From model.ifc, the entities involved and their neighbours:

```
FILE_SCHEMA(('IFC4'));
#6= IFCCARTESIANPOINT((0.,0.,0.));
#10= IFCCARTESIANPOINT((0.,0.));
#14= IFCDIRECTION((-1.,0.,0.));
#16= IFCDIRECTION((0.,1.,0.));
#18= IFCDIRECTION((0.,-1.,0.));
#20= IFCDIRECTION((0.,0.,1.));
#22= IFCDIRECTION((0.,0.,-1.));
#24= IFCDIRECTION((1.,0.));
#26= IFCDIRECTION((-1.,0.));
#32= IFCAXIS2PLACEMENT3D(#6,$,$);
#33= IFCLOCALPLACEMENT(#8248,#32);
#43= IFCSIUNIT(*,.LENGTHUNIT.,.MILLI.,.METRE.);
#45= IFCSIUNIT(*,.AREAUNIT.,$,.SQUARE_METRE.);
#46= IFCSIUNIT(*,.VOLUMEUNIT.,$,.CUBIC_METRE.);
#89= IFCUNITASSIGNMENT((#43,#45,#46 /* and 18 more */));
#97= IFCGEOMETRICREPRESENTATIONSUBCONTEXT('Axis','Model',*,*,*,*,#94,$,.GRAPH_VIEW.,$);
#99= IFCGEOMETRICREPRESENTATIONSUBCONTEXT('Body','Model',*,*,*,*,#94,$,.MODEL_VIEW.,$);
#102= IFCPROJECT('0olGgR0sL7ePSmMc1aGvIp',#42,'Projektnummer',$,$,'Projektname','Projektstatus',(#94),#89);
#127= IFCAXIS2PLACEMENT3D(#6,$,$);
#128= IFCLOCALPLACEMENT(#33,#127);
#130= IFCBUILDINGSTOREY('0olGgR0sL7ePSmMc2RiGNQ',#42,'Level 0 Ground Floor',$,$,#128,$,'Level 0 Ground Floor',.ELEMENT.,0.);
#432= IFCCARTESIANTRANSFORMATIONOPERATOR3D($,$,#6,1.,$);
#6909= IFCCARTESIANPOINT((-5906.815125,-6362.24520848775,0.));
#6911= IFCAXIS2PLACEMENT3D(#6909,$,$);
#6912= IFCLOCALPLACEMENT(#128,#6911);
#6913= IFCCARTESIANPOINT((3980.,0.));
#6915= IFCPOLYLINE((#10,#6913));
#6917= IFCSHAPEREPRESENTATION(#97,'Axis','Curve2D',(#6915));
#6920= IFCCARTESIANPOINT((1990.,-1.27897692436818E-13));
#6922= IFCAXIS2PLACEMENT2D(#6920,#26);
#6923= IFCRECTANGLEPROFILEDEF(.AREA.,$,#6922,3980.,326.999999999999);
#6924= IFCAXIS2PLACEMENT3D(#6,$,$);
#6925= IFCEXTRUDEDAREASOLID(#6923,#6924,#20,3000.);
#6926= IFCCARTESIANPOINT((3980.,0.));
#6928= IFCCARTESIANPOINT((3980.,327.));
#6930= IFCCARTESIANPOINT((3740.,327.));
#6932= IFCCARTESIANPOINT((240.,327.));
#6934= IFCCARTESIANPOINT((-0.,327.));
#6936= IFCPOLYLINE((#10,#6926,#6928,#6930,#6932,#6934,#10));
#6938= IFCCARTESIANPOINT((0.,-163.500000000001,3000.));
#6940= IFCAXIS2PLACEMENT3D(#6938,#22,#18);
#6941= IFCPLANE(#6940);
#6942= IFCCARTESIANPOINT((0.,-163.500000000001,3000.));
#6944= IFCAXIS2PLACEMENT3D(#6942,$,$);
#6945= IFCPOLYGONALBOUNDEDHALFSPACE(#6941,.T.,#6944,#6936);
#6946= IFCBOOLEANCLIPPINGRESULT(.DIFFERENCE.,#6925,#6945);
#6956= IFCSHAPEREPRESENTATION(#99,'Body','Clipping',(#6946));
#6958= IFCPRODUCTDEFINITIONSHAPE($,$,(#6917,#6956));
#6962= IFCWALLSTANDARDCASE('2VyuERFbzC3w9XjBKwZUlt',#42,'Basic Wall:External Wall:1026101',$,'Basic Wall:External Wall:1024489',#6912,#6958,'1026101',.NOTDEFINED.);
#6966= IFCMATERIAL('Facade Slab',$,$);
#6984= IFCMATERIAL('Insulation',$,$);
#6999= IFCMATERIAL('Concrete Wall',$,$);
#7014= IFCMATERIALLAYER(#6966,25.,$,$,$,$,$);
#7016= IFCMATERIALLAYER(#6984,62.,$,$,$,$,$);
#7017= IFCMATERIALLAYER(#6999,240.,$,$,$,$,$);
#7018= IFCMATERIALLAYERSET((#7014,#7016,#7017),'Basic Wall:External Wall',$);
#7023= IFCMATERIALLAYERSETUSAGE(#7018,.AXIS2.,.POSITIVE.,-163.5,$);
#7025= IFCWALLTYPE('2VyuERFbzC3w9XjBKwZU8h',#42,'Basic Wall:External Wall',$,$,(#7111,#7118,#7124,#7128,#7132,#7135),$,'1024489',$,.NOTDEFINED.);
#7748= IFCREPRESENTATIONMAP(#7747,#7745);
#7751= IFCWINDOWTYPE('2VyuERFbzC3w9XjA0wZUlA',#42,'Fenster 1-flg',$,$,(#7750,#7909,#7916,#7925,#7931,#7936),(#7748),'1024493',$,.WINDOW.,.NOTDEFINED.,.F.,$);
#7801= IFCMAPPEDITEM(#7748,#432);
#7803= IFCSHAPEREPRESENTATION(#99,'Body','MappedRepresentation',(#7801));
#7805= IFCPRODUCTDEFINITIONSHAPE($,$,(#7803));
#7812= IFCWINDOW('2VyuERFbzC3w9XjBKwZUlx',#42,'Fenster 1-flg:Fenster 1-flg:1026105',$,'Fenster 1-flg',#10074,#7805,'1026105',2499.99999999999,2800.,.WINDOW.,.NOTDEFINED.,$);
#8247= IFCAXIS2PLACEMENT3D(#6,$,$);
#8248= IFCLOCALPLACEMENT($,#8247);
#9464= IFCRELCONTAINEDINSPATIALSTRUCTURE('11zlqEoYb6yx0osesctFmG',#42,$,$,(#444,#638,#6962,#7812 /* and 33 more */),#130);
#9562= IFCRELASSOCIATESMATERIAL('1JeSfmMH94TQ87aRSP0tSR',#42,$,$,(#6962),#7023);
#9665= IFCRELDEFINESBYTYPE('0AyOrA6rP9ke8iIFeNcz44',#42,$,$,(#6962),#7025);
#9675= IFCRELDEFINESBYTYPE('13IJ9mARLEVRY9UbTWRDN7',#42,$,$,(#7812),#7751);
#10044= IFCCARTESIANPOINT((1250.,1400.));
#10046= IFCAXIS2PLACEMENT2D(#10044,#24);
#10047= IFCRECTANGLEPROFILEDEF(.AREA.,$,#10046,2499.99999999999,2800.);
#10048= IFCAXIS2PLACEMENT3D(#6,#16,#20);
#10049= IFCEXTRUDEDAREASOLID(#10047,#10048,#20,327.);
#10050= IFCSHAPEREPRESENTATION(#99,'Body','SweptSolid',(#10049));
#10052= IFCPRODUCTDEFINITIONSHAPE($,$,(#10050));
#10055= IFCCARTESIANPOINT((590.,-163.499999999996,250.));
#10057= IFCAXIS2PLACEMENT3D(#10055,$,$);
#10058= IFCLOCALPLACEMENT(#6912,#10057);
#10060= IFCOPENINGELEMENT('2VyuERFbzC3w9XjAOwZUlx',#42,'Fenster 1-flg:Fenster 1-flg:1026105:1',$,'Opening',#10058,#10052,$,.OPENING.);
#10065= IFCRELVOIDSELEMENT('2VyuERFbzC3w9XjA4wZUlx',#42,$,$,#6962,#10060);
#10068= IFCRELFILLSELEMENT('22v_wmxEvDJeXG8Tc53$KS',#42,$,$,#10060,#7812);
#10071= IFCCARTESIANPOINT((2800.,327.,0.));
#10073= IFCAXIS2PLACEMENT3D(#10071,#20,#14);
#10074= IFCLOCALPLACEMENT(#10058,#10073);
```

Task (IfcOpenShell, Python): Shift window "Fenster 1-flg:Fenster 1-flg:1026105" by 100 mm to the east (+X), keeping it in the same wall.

```python
import ifcopenshell
import ifcopenshell.api.geometry
import ifcopenshell.util.placement

model = ifcopenshell.open("model.ifc")

window = model.by_guid("2VyuERFbzC3w9XjBKwZUlx")
opening = window.FillsVoids[0].RelatingOpeningElement
wall = opening.VoidsElements[0].RelatingBuildingElement

wall_matrix = ifcopenshell.util.placement.get_local_placement(wall.ObjectPlacement)
shift = wall_matrix[:3, 0] * 100.0
before = ifcopenshell.util.placement.get_local_placement(window.ObjectPlacement)[:3, 3].copy()

# The window is placed relative to its opening, so it follows when the opening moves.
matrix = ifcopenshell.util.placement.get_local_placement(opening.ObjectPlacement)
matrix[:3, 3] += shift
ifcopenshell.api.geometry.edit_object_placement(
    model, product=opening, matrix=matrix, is_si=False, should_transform_children=True
)

after = ifcopenshell.util.placement.get_local_placement(window.ObjectPlacement)[:3, 3]
print("window moved by", (after - before).round(3) + 0.0)

model.write("model_updated.ifc")
```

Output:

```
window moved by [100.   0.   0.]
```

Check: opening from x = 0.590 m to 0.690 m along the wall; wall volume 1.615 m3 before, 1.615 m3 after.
